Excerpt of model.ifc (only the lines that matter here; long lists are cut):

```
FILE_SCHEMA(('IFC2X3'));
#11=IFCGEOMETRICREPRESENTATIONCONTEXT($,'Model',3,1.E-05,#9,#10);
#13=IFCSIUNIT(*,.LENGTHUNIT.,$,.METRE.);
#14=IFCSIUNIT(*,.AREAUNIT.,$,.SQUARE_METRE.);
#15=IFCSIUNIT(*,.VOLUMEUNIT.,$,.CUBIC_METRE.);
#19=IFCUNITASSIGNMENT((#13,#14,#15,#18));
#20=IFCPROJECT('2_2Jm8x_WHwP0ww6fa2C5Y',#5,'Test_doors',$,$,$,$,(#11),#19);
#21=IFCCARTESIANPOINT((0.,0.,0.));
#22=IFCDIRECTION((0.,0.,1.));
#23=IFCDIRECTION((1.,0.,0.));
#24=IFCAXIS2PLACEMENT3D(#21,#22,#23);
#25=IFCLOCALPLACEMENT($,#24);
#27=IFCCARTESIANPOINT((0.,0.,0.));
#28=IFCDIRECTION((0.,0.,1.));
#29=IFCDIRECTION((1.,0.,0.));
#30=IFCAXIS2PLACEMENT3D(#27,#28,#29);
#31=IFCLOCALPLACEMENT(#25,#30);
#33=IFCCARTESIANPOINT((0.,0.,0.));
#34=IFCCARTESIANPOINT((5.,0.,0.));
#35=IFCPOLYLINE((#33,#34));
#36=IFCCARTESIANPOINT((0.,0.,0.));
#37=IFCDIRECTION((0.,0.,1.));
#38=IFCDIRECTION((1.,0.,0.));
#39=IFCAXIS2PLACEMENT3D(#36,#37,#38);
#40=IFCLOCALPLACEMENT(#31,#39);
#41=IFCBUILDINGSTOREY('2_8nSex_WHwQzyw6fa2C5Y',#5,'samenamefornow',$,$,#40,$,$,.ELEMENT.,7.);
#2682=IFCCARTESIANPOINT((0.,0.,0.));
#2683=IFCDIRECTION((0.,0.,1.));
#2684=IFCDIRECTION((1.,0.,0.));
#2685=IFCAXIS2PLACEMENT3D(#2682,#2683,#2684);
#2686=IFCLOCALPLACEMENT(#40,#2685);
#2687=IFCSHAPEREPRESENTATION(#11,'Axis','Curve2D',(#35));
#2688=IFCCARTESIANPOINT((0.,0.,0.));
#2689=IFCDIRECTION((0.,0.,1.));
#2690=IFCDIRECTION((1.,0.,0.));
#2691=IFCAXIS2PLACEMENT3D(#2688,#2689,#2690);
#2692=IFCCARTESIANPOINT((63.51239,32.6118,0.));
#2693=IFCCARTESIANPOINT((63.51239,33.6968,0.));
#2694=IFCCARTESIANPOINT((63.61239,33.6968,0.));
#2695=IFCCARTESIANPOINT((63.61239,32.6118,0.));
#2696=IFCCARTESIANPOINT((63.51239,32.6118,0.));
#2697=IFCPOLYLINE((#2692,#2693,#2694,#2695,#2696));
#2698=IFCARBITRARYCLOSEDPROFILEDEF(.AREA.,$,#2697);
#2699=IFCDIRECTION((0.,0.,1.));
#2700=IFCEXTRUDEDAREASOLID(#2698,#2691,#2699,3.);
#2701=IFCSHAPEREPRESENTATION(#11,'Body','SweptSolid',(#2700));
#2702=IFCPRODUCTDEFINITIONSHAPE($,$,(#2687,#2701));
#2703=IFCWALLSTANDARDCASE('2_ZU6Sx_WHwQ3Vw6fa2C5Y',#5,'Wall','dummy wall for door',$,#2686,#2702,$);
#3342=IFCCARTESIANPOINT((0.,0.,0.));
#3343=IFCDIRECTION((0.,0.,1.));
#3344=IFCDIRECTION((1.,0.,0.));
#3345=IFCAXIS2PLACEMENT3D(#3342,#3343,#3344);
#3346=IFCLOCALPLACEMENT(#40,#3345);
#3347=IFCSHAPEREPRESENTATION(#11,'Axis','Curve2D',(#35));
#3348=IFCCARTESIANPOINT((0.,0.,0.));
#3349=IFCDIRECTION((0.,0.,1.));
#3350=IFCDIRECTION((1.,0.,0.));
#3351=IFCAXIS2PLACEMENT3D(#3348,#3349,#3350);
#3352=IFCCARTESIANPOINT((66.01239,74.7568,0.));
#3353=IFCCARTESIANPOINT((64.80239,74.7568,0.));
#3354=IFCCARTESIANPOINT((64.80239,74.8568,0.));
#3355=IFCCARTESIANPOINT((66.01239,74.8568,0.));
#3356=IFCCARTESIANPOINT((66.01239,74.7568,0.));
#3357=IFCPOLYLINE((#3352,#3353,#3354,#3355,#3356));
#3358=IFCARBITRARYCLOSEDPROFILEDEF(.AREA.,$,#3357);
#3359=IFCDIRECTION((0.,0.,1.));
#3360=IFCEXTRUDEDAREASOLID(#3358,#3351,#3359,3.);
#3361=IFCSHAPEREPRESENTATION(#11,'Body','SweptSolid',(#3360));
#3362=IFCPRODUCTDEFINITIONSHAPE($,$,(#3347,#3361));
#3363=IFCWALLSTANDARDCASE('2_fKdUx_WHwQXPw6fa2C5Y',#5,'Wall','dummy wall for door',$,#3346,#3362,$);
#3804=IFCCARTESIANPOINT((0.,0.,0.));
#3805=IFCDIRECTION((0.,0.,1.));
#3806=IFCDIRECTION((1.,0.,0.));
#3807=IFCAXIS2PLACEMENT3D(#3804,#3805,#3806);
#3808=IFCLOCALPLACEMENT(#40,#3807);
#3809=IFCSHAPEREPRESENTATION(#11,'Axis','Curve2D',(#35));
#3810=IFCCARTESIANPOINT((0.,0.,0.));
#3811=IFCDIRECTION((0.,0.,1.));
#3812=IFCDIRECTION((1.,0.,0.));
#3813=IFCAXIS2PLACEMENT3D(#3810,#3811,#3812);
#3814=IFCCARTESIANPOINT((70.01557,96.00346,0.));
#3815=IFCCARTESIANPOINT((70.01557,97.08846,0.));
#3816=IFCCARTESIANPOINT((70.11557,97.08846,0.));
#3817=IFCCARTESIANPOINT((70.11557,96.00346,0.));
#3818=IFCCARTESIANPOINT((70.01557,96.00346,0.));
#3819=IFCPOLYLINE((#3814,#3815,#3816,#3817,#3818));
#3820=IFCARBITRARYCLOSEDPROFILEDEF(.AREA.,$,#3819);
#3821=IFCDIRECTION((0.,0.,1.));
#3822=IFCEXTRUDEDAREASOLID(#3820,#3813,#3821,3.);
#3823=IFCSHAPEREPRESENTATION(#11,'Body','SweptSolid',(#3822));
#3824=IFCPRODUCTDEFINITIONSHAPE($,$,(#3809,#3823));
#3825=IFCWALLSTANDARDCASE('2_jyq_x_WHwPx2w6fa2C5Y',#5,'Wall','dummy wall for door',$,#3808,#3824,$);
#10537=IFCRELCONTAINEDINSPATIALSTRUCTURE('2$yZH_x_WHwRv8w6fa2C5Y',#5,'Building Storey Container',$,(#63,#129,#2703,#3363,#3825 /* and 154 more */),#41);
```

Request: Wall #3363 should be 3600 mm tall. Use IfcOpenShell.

```python
import ifcopenshell
import ifcopenshell.geom
import ifcopenshell.util.shape
import ifcopenshell.util.unit

model = ifcopenshell.open("model.ifc")
unit_scale = ifcopenshell.util.unit.calculate_unit_scale(model)
settings = ifcopenshell.geom.settings()


def volume(element):
    """Net volume in cubic metres, openings subtracted."""
    shape = ifcopenshell.geom.create_shape(settings, element)
    return ifcopenshell.util.shape.get_volume(shape.geometry)


wall = model.by_guid("2_fKdUx_WHwQXPw6fa2C5Y")
before = volume(wall)

body = next(r for r in wall.Representation.Representations if r.RepresentationIdentifier == "Body")
solid = body.Items[0]
old_height = solid.Depth
solid.Depth = 3.6 / unit_scale
after = volume(wall)

print(f"height {old_height:g} -> {solid.Depth:g}, volume {before:.3f} -> {after:.3f} m3")

model.write("model_v2.ifc")
```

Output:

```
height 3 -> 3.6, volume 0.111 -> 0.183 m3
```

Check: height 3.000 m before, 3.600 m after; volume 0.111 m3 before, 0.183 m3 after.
